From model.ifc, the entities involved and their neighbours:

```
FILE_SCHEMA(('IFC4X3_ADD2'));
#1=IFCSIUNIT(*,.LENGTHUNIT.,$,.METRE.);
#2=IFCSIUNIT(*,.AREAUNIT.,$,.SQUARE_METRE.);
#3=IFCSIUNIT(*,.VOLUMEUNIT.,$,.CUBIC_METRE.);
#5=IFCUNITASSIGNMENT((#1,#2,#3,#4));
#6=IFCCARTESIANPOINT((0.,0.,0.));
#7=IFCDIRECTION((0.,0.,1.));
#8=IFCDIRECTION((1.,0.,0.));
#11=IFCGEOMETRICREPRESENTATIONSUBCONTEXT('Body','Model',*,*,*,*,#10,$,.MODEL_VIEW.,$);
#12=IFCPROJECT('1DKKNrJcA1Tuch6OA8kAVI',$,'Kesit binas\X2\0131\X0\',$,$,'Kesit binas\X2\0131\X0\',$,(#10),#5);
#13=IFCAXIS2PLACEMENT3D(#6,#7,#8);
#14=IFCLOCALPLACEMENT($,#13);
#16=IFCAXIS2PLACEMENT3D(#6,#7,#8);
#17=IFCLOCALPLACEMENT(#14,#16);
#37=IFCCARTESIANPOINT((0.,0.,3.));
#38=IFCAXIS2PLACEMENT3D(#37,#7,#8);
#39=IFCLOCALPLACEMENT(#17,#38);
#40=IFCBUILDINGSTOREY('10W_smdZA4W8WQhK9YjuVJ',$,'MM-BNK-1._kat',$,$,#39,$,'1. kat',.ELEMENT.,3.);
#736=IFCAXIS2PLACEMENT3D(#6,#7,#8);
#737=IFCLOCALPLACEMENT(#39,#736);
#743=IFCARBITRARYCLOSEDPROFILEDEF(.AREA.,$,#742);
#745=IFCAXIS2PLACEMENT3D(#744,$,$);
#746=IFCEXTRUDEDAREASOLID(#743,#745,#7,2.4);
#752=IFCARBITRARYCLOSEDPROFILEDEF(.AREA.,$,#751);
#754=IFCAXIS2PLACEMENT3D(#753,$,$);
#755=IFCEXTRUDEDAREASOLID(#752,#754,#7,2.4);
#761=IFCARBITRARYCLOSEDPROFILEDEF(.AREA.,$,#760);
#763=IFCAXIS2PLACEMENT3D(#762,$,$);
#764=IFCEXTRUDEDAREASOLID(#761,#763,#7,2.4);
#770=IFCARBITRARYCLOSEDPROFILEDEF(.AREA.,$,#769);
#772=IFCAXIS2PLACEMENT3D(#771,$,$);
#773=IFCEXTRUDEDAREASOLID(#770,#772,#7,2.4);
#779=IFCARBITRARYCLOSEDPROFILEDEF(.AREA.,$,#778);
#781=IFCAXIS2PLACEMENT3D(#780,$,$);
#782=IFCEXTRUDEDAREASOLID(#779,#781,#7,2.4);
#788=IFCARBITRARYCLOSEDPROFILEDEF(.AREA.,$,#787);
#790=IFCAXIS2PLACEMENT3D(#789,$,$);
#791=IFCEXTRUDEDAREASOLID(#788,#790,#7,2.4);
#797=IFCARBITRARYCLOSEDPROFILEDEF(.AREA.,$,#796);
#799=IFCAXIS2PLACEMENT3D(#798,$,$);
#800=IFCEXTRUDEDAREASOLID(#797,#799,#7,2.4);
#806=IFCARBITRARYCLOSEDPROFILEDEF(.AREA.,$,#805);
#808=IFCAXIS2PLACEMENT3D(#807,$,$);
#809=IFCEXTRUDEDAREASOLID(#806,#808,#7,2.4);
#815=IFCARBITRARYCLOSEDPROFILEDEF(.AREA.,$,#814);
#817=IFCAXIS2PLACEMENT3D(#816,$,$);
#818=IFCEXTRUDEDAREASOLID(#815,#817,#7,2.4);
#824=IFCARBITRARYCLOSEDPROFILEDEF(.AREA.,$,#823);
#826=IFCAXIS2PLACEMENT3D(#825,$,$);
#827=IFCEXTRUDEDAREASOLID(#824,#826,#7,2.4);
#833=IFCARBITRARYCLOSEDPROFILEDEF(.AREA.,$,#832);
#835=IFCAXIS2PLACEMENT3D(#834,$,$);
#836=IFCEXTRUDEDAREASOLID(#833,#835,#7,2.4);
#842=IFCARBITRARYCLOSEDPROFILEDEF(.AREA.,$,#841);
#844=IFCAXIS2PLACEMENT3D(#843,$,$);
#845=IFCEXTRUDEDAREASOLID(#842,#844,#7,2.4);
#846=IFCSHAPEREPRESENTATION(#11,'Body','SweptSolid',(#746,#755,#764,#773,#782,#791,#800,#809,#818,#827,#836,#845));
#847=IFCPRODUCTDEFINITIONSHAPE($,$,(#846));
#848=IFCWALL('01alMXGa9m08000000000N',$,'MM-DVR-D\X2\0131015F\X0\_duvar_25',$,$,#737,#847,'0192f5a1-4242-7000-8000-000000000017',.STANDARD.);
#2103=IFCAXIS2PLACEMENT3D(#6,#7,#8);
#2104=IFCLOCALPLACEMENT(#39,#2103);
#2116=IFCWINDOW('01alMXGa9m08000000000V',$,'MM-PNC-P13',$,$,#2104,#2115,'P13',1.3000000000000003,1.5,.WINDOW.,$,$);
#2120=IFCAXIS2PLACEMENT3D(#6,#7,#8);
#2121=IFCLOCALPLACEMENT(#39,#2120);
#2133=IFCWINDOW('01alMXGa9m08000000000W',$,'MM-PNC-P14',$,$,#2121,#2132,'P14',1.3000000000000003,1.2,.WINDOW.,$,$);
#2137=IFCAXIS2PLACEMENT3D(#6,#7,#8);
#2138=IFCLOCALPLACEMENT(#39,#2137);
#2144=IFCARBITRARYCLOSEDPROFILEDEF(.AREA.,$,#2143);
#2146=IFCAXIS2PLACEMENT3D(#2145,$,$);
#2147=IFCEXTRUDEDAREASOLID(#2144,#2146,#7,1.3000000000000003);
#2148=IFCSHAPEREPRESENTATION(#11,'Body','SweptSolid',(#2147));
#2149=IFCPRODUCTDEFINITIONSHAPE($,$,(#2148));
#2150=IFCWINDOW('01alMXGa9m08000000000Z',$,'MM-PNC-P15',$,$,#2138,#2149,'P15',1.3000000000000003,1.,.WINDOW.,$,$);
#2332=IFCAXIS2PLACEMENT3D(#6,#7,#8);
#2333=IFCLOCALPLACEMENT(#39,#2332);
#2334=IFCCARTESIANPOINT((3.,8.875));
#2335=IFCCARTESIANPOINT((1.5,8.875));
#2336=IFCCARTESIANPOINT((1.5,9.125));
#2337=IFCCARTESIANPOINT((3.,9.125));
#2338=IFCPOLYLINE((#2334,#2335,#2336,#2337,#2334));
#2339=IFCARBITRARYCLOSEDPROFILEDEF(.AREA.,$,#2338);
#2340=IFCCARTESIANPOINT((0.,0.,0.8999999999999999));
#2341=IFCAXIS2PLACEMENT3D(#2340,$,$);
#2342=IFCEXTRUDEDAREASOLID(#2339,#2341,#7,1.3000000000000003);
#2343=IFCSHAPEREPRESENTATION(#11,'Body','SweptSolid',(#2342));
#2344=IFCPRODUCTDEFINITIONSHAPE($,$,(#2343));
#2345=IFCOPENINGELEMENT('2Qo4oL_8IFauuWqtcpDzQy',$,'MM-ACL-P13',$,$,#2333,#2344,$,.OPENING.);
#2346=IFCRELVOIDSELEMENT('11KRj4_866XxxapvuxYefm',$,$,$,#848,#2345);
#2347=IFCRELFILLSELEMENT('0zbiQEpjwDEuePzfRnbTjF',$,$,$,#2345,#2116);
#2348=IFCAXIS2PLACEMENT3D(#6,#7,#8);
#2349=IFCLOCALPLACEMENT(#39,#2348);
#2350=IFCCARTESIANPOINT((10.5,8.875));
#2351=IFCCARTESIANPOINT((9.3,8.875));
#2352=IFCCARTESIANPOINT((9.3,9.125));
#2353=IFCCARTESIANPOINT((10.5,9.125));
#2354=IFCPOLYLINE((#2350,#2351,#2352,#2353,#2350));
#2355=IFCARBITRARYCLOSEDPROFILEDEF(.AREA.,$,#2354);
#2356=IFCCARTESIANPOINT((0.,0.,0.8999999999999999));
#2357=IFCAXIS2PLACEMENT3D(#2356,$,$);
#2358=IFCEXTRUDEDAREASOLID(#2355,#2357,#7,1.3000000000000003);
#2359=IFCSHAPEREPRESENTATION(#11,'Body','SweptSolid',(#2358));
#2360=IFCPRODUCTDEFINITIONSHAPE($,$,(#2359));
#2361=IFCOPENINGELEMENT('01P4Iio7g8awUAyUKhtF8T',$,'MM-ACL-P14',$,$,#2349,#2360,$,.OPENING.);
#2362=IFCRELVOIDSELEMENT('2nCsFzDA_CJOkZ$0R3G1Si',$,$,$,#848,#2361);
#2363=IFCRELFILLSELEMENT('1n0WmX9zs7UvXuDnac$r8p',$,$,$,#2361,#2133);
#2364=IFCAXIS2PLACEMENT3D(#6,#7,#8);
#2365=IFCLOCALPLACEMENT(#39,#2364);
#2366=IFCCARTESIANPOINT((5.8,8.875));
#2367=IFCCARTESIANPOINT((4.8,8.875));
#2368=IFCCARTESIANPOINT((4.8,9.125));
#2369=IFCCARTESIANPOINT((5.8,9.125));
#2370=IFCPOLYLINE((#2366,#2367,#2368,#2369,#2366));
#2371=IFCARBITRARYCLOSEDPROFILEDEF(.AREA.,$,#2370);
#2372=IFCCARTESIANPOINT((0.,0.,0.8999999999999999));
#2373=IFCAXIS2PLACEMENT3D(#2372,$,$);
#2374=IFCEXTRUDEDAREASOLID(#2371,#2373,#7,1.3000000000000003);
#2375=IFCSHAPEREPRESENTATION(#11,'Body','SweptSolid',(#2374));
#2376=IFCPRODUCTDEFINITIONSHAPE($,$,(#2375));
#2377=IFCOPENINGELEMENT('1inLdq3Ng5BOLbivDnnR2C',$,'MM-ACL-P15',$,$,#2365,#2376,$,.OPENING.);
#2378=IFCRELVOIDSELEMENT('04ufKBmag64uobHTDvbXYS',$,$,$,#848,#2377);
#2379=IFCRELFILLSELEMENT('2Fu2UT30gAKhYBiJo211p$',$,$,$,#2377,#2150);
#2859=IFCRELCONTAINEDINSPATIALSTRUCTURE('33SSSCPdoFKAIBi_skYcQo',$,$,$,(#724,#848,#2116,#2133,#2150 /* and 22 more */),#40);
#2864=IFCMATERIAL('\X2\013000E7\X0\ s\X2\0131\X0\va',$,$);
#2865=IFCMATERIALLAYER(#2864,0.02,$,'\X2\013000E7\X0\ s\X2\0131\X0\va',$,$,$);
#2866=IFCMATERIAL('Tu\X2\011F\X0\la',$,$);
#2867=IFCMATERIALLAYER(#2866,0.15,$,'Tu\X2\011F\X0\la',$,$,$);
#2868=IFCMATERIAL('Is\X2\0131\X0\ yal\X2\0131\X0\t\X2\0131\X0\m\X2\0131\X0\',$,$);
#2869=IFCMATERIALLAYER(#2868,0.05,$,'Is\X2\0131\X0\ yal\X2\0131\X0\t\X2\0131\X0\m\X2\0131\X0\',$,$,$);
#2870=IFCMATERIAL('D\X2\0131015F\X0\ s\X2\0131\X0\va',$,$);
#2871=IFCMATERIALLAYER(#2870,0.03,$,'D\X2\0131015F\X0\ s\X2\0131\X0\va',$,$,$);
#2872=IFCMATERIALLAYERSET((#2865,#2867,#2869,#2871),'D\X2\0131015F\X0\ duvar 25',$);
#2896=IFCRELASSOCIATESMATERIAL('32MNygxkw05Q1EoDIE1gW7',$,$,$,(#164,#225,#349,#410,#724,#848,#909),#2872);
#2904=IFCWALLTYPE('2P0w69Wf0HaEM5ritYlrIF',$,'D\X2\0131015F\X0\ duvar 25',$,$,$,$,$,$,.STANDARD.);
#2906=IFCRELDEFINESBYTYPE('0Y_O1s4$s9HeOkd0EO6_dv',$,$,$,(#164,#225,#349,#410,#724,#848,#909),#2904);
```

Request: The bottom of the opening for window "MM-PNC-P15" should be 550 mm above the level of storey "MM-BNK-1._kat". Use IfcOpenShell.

```python
import numpy as np
import ifcopenshell
import ifcopenshell.api.geometry
import ifcopenshell.geom
import ifcopenshell.util.element
import ifcopenshell.util.placement
import ifcopenshell.util.shape
import ifcopenshell.util.unit

model = ifcopenshell.open("model.ifc")
unit_scale = ifcopenshell.util.unit.calculate_unit_scale(model)

window = model.by_id(2150)
opening = window.FillsVoids[0].RelatingOpeningElement
storey = ifcopenshell.util.element.get_container(window, ifc_class="IfcBuildingStorey")
level = ifcopenshell.util.placement.get_local_placement(storey.ObjectPlacement)[2, 3]

# The opening's origin need not be at the sill, so measure its lowest point.
shape = ifcopenshell.geom.create_shape(ifcopenshell.geom.settings(), opening)
bottom = ifcopenshell.util.shape.get_shape_bottom_elevation(shape, shape.geometry) / unit_scale
dz = level + 0.55 - bottom

shift = np.array([0.0, 0.0, dz])
# The window is not placed relative to its opening, so move both.
for product in (opening, window):
    matrix = ifcopenshell.util.placement.get_local_placement(product.ObjectPlacement)
    matrix[:3, 3] += shift
    ifcopenshell.api.geometry.edit_object_placement(model, product=product, matrix=matrix, is_si=False)

print(f"moved by {dz * unit_scale:+.3f} m")

model.write("model_edited.ifc")
```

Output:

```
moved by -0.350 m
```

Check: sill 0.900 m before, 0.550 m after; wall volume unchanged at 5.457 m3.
